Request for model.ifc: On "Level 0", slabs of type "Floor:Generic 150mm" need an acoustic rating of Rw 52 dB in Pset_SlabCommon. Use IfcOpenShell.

First a look at what the model holds.

```python
import ifcopenshell
import ifcopenshell.util.element

model = ifcopenshell.open("model.ifc")
print(model.schema)
storey = next(s for s in model.by_type("IfcBuildingStorey") if s.Name == "Level 0")
slabs = [e for e in ifcopenshell.util.element.get_decomposition(storey) if e.is_a("IfcSlab")]
seen = {}
for e in slabs:
    element_type = ifcopenshell.util.element.get_type(e)
    key = (element_type.Name if element_type != e and element_type else None, ifcopenshell.util.element.get_pset(e, "Pset_SlabCommon", "AcousticRating"))
    seen[key] = seen.get(key, 0) + 1
for (name, value), count in sorted(seen.items(), key=str):
    print(count, "x", name, "|", value)
```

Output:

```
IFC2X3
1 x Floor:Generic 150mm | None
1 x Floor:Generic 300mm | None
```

```python
import ifcopenshell
import ifcopenshell.api.pset
import ifcopenshell.util.element

model = ifcopenshell.open("model.ifc")

storey = next(s for s in model.by_type("IfcBuildingStorey") if s.Name == "Level 0")
slabs = [e for e in ifcopenshell.util.element.get_decomposition(storey) if e.is_a("IfcSlab")]

count = 0
for e in slabs:
    element_type = ifcopenshell.util.element.get_type(e)
    if element_type in (None, e) or element_type.Name != "Floor:Generic 150mm":
        continue
    # add_pset returns the element's existing set when there is one.
    pset = ifcopenshell.api.pset.add_pset(model, product=e, name="Pset_SlabCommon")
    ifcopenshell.api.pset.edit_pset(model, pset=pset, properties={"AcousticRating": "Rw 52 dB"})
    count += 1

print(count, "slabs updated")

model.write("model-out.ifc")
```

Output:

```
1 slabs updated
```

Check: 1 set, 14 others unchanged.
